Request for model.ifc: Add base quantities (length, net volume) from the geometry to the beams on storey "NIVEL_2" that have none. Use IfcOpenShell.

First a look at what the model holds.

```python
import ifcopenshell
import ifcopenshell.util.element
import ifcopenshell.util.unit

model = ifcopenshell.open("model.ifc")
print(model.schema)
for unit_type in ("LENGTHUNIT", "AREAUNIT", "VOLUMEUNIT"):
    print(unit_type, ifcopenshell.util.unit.calculate_unit_scale(model, unit_type))
storey = next(s for s in model.by_type("IfcBuildingStorey") if s.Name == "NIVEL_2")
beams = [e for e in ifcopenshell.util.element.get_decomposition(storey) if e.is_a("IfcBeam")]
for e in sorted(beams, key=lambda e: e.id()):
    print(e.id(), e.is_a(), e.Name, list(ifcopenshell.util.element.get_psets(e, qtos_only=True)), sep=" | ")
```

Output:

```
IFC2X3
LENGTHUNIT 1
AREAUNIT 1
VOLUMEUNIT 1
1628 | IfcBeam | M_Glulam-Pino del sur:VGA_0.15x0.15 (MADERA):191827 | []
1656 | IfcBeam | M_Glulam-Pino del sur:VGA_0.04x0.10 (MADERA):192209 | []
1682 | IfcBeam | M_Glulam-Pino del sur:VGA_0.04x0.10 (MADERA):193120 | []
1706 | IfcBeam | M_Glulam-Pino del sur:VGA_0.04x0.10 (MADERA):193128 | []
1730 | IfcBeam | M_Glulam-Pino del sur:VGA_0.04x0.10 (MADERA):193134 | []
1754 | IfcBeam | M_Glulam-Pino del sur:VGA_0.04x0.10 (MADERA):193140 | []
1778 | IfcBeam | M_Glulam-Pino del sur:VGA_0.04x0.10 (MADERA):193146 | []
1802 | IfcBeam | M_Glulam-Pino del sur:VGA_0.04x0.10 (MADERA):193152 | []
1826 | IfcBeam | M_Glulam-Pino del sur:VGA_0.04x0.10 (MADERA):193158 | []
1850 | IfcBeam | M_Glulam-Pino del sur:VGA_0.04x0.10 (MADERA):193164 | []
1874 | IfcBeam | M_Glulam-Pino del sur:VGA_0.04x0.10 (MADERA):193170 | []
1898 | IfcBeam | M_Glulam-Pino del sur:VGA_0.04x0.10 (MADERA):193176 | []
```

```python
import ifcopenshell
import ifcopenshell.api.pset
import ifcopenshell.geom
import ifcopenshell.util.element
import ifcopenshell.util.shape
import ifcopenshell.util.unit

model = ifcopenshell.open("model.ifc")
unit_scale = ifcopenshell.util.unit.calculate_unit_scale(model)
volume_scale = ifcopenshell.util.unit.calculate_unit_scale(model, "VOLUMEUNIT")
settings = ifcopenshell.geom.settings()

storey = next(s for s in model.by_type("IfcBuildingStorey") if s.Name == "NIVEL_2")
beams = [e for e in ifcopenshell.util.element.get_decomposition(storey) if e.is_a("IfcBeam")]

for e in sorted(beams, key=lambda e: e.id()):
    if ifcopenshell.util.element.get_psets(e, qtos_only=True, should_inherit=False):
        continue
    # Geometry comes back in metres, in the element's own axes.
    shape = ifcopenshell.geom.create_shape(settings, e)
    values = {
        "Length": ifcopenshell.util.shape.get_max_xyz(shape.geometry) / unit_scale,
        "NetVolume": ifcopenshell.util.shape.get_volume(shape.geometry) / volume_scale,
    }
    qto = ifcopenshell.api.pset.add_qto(model, product=e, name="BaseQuantities")
    ifcopenshell.api.pset.edit_qto(model, qto=qto, properties=values)
    print(e.id(), {k: round(v, 3) for k, v in values.items()})

model.write("model-out.ifc")
```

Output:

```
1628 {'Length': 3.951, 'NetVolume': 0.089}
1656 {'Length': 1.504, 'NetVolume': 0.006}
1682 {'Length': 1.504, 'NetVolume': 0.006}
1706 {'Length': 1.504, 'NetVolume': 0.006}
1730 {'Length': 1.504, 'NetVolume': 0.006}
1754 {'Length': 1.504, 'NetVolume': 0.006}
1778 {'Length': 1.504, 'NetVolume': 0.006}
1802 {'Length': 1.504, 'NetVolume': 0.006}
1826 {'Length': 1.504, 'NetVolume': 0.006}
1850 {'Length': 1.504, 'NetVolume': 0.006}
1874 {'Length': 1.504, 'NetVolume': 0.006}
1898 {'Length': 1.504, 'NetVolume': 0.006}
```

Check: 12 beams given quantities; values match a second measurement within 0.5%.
